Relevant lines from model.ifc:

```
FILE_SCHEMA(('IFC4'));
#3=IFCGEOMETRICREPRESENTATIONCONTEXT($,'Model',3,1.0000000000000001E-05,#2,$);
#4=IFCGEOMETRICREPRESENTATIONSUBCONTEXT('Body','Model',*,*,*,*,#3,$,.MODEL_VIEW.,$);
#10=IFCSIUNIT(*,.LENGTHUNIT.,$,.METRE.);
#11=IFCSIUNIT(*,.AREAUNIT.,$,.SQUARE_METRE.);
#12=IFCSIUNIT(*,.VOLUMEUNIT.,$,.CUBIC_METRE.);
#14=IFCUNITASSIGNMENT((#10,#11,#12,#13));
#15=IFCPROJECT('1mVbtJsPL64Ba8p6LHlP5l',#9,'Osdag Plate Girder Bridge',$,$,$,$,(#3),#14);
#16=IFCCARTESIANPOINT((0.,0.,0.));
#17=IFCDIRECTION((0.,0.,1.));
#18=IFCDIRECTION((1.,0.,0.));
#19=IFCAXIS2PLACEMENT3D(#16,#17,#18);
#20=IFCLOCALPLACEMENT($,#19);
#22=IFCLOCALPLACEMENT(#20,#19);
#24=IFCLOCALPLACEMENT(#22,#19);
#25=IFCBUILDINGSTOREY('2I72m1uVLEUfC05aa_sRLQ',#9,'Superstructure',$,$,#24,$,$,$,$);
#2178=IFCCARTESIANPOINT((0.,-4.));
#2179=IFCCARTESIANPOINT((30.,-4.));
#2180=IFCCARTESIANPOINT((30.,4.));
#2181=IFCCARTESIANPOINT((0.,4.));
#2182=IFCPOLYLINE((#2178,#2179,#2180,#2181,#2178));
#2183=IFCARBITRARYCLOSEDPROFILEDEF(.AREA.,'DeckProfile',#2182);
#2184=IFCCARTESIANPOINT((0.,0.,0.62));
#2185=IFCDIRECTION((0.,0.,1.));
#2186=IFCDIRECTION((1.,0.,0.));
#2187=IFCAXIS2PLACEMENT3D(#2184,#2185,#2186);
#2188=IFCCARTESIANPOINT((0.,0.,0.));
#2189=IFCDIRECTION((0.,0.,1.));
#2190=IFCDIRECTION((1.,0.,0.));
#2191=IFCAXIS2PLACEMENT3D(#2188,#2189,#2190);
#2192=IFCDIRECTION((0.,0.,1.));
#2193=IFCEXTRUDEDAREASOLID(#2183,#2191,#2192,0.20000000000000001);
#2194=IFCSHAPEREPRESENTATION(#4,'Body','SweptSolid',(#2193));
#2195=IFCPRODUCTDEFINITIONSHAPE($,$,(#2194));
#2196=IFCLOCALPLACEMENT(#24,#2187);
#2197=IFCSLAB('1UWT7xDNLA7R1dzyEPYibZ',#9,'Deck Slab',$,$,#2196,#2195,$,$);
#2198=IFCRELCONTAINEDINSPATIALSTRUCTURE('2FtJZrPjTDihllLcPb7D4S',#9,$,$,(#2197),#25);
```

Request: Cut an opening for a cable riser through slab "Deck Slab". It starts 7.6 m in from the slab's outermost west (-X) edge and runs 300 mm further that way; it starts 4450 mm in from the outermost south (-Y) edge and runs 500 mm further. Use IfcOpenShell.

```python
import numpy as np
import ifcopenshell
import ifcopenshell.api.feature
import ifcopenshell.api.geometry
import ifcopenshell.api.root
import ifcopenshell.geom
import ifcopenshell.util.placement
import ifcopenshell.util.representation
import ifcopenshell.util.shape
import ifcopenshell.util.unit

model = ifcopenshell.open("model.ifc")
unit_scale = ifcopenshell.util.unit.calculate_unit_scale(model)
settings = ifcopenshell.geom.settings()


def volume(element):
    """Net volume in cubic metres, openings subtracted."""
    shape = ifcopenshell.geom.create_shape(settings, element)
    return ifcopenshell.util.shape.get_volume(shape.geometry)


slab = model.by_guid("1UWT7xDNLA7R1dzyEPYibZ")
before = volume(slab)

# Extent in the slab's own axes, in metres. The edges named are its -X and -Y sides.
slab_shape = ifcopenshell.geom.create_shape(settings, slab)
vertices = ifcopenshell.util.shape.get_vertices(slab_shape.geometry)
x_min, y_min, bottom = vertices.min(axis=0)
top = vertices[:, 2].max()

opening = ifcopenshell.api.root.create_entity(model, ifc_class="IfcOpeningElement", name="Cable riser opening", predefined_type="OPENING")
context = ifcopenshell.util.representation.get_context(model, "Model", "Body", "MODEL_VIEW")
width, depth = 0.3, 0.5
outline = [(0.0, 0.0), (width, 0.0), (width, depth), (0.0, depth), (0.0, 0.0)]
# Overshoot both faces by 50 mm so the cut is clean.
shape = ifcopenshell.api.geometry.add_slab_representation(
    model, context=context, depth=top - bottom + 0.1, polyline=outline
)
ifcopenshell.api.geometry.assign_representation(model, product=opening, representation=shape)

matrix = ifcopenshell.util.placement.get_local_placement(slab.ObjectPlacement)
matrix[:, 3] = matrix @ np.append(np.array([x_min + 7.6, y_min + 4.45, bottom - 0.05]) / unit_scale, 1.0)
ifcopenshell.api.geometry.edit_object_placement(model, product=opening, matrix=matrix, is_si=False)
ifcopenshell.api.feature.add_feature(model, feature=opening, element=slab)

after = volume(slab)

print(f"slab volume {before:.3f} -> {after:.3f} m3")

model.write("model_v2.ifc")
```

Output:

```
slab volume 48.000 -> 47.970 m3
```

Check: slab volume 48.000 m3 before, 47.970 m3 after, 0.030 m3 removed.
